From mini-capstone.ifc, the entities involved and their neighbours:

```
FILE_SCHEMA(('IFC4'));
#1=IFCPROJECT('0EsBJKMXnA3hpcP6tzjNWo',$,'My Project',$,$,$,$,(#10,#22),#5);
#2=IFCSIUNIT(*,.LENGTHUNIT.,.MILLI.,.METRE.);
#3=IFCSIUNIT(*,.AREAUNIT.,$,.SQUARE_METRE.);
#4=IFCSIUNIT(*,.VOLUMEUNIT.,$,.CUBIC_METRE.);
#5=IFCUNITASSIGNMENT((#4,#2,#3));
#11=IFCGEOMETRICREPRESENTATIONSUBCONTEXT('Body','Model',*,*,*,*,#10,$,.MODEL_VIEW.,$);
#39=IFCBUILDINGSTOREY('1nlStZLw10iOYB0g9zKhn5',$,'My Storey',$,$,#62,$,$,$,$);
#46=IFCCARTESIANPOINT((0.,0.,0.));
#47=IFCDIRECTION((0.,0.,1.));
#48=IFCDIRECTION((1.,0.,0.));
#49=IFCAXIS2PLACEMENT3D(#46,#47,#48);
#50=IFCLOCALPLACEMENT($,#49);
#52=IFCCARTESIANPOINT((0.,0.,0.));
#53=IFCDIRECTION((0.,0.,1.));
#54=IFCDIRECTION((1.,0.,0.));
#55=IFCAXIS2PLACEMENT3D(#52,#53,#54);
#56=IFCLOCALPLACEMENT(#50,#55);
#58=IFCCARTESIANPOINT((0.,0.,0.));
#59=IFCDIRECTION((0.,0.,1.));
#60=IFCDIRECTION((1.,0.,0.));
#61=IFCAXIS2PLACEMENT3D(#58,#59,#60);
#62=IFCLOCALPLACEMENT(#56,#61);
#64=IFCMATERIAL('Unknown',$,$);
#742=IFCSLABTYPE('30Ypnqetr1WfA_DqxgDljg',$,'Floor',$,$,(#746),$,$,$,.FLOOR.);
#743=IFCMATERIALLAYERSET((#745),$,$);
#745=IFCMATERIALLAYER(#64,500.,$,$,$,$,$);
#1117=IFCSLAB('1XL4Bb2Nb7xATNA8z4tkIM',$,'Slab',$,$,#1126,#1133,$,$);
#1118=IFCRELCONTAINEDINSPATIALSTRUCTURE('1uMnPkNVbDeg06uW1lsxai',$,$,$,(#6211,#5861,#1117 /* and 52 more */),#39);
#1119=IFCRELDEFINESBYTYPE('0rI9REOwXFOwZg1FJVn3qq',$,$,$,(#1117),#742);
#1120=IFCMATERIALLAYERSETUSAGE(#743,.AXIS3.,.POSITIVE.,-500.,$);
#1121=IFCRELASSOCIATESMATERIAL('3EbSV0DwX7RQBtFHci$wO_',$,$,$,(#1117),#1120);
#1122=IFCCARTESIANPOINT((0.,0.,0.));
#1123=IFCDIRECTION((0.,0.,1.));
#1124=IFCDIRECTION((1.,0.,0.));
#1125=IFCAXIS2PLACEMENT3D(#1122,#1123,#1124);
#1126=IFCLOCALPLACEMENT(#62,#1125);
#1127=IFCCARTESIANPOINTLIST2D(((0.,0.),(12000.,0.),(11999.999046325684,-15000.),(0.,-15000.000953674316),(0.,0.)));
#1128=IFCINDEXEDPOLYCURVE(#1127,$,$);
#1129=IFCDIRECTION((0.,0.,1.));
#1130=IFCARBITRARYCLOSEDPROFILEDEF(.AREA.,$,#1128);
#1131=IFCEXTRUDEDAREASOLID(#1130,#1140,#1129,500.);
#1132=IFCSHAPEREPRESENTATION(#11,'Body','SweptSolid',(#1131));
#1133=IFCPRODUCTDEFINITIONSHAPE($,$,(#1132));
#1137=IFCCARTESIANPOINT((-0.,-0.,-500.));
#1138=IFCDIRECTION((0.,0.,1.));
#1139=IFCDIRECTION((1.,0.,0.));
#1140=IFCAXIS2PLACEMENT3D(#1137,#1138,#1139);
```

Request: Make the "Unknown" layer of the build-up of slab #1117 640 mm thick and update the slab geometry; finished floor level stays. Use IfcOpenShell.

```python
import ifcopenshell
import ifcopenshell.util.element
import ifcopenshell.util.representation

model = ifcopenshell.open("mini-capstone.ifc")

layer_set = model.by_id(743)
layer = next(l for l in layer_set.MaterialLayers if l.Material and l.Material.Name == "Unknown")
change = 640.0 - layer.LayerThickness
layer.LayerThickness += change

# Geometry does not follow the layer set by itself.
slabs = [e for e in ifcopenshell.util.element.get_elements_by_material(model, layer_set) if e.is_a("IfcSlab")]
for slab in sorted(slabs, key=lambda e: e.id()):
    body = ifcopenshell.util.representation.get_representation(slab, "Model", "Body")
    solid = body.Items[0]
    old_depth = solid.Depth
    solid.Depth += change
    # Extruded upwards: lower the start of the extrusion so the top stays.
    x, y, z = solid.Position.Location.Coordinates
    solid.Position.Location = model.createIfcCartesianPoint((x, y, z - change))
    print(slab.id(), f"{old_depth:g} -> {solid.Depth:g}")

# The layers are counted up from the underside, which has moved.
for usage in {ifcopenshell.util.element.get_material(slab) for slab in slabs}:
    usage.OffsetFromReferenceLine -= change

model.write("mini-capstone-out.ifc")
```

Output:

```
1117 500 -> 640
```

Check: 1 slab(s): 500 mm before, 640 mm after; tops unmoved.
